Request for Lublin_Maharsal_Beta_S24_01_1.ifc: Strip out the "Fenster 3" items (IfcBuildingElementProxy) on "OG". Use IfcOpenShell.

First a look at what the model holds.

```python
import ifcopenshell
import ifcopenshell.util.element

model = ifcopenshell.open("Lublin_Maharsal_Beta_S24_01_1.ifc")
print(model.schema)
storey = next(s for s in model.by_type("IfcBuildingStorey") if s.Name == "OG")
proxies = [e for e in ifcopenshell.util.element.get_decomposition(storey) if e.is_a("IfcBuildingElementProxy")]
seen = {}
for e in proxies:
    element_type = ifcopenshell.util.element.get_type(e)
    name = element_type.Name if element_type not in (None, e) else None
    seen[name] = seen.get(name, 0) + 1
for name, count in sorted(seen.items(), key=str):
    print(count, "x", name)
```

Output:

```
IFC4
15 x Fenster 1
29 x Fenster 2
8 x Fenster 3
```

```python
import ifcopenshell
import ifcopenshell.api.root
import ifcopenshell.util.element

model = ifcopenshell.open("Lublin_Maharsal_Beta_S24_01_1.ifc")

storey = next(s for s in model.by_type("IfcBuildingStorey") if s.Name == "OG")
proxies = [e for e in ifcopenshell.util.element.get_decomposition(storey) if e.is_a("IfcBuildingElementProxy")]
targets = [e for e in proxies if (t := ifcopenshell.util.element.get_type(e)) not in (None, e) and t.Name == "Fenster 3"]

for e in targets:
    ifcopenshell.api.root.remove_product(model, product=e)
print(len(targets), "removed")

model.write("Lublin_Maharsal_Beta_S24_01_1-out.ifc")
```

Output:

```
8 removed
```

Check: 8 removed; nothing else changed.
